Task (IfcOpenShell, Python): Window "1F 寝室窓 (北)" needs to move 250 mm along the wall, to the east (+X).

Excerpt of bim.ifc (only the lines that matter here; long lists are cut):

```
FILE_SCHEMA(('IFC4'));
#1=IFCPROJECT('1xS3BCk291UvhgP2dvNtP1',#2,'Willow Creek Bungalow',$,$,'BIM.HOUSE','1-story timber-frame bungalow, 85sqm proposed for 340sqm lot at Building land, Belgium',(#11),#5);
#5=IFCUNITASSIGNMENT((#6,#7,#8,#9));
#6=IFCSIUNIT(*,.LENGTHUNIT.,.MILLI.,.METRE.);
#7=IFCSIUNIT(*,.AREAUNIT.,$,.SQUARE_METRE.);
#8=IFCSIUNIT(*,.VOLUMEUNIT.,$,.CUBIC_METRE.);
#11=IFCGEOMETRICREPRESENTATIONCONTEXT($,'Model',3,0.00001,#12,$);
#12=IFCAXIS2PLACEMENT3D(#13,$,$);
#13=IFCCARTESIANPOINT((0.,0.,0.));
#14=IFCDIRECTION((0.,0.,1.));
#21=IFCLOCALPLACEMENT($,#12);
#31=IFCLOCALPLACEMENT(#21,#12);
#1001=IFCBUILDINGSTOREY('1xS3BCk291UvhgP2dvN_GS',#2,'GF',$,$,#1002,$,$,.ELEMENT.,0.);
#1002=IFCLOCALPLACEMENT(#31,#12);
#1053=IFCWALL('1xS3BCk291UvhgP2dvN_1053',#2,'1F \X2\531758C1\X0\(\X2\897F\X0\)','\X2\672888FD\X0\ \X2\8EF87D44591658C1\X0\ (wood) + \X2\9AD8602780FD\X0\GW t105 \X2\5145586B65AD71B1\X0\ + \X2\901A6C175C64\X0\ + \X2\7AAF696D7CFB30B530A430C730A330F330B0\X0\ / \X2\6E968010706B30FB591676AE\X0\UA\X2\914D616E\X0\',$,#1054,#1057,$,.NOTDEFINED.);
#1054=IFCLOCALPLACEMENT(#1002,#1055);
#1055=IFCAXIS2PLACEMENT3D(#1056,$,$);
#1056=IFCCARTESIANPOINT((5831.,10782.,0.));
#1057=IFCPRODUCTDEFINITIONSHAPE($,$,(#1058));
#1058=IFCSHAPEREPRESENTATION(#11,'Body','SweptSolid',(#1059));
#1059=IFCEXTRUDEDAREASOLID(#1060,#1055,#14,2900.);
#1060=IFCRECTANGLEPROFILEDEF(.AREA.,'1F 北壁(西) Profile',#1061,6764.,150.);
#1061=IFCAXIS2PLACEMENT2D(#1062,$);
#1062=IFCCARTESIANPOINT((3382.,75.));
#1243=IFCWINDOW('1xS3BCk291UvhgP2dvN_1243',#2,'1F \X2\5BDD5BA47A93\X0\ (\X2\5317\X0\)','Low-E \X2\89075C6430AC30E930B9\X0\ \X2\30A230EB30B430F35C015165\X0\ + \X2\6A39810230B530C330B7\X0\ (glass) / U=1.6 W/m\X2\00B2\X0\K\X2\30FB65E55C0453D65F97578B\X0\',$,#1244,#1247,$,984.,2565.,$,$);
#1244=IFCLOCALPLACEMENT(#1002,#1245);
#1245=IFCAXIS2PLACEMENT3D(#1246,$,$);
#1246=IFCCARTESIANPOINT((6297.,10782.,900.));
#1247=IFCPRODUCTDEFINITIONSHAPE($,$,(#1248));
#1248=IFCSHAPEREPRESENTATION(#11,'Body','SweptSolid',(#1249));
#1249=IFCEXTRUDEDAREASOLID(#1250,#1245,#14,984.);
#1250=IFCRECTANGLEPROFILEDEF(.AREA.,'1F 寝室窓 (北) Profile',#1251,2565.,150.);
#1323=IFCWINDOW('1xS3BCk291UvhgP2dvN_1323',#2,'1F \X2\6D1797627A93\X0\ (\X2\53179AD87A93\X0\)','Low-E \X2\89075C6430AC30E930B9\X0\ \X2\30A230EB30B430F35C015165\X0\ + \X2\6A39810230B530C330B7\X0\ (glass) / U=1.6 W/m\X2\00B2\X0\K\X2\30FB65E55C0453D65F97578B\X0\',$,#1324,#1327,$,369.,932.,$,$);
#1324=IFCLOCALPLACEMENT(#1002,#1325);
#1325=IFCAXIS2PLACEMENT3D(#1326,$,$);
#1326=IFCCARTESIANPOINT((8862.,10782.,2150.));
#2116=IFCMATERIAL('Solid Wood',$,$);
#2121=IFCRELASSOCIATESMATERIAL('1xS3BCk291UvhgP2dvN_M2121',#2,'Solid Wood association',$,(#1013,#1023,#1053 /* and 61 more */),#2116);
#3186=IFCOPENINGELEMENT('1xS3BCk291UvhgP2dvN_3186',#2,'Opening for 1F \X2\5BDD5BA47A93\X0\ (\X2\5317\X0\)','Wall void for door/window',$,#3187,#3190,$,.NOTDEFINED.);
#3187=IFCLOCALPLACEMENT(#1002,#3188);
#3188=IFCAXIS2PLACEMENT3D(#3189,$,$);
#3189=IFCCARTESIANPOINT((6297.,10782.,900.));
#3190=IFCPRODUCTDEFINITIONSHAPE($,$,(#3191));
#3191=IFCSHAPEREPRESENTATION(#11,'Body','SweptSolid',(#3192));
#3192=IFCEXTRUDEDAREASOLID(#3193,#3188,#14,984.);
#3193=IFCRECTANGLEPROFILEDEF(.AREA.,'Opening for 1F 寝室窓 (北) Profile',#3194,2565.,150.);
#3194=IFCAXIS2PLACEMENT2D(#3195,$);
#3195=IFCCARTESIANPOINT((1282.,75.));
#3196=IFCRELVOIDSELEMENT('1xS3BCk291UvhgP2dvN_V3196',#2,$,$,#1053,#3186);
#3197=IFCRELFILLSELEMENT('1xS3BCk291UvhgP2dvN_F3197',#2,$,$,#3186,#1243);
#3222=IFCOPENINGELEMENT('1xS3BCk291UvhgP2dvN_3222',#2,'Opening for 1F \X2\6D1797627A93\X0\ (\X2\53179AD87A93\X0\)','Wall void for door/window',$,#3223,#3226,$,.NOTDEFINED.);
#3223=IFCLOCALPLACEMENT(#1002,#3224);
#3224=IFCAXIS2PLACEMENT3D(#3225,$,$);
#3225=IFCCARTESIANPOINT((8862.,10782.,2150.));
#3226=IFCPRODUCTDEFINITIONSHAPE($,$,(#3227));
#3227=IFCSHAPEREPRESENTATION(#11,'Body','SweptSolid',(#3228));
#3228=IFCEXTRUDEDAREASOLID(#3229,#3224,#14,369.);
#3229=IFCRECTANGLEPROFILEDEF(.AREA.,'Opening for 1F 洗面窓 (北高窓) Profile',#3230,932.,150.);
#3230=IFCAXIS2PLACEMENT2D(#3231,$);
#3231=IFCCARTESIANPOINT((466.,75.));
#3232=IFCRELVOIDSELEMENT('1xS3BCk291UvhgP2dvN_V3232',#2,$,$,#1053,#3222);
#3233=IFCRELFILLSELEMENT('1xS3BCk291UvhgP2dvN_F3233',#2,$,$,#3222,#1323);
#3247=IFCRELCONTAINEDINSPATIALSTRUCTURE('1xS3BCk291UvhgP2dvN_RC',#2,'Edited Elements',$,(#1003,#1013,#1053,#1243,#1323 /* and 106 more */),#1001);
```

```python
import ifcopenshell
import ifcopenshell.api.geometry
import ifcopenshell.util.placement

model = ifcopenshell.open("bim.ifc")

window = model.by_guid("1xS3BCk291UvhgP2dvN_1243")
opening = window.FillsVoids[0].RelatingOpeningElement
wall = opening.VoidsElements[0].RelatingBuildingElement

wall_matrix = ifcopenshell.util.placement.get_local_placement(wall.ObjectPlacement)
shift = wall_matrix[:3, 0] * 250.0
before = ifcopenshell.util.placement.get_local_placement(window.ObjectPlacement)[:3, 3].copy()

# The window is not placed relative to its opening, so move both.
for product in (opening, window):
    matrix = ifcopenshell.util.placement.get_local_placement(product.ObjectPlacement)
    matrix[:3, 3] += shift
    ifcopenshell.api.geometry.edit_object_placement(model, product=product, matrix=matrix, is_si=False)

after = ifcopenshell.util.placement.get_local_placement(window.ObjectPlacement)[:3, 3]
print("window moved by", (after - before).round(3) + 0.0)

model.write("bim_updated.ifc")
```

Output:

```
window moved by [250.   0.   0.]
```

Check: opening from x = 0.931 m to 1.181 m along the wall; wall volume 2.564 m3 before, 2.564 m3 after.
